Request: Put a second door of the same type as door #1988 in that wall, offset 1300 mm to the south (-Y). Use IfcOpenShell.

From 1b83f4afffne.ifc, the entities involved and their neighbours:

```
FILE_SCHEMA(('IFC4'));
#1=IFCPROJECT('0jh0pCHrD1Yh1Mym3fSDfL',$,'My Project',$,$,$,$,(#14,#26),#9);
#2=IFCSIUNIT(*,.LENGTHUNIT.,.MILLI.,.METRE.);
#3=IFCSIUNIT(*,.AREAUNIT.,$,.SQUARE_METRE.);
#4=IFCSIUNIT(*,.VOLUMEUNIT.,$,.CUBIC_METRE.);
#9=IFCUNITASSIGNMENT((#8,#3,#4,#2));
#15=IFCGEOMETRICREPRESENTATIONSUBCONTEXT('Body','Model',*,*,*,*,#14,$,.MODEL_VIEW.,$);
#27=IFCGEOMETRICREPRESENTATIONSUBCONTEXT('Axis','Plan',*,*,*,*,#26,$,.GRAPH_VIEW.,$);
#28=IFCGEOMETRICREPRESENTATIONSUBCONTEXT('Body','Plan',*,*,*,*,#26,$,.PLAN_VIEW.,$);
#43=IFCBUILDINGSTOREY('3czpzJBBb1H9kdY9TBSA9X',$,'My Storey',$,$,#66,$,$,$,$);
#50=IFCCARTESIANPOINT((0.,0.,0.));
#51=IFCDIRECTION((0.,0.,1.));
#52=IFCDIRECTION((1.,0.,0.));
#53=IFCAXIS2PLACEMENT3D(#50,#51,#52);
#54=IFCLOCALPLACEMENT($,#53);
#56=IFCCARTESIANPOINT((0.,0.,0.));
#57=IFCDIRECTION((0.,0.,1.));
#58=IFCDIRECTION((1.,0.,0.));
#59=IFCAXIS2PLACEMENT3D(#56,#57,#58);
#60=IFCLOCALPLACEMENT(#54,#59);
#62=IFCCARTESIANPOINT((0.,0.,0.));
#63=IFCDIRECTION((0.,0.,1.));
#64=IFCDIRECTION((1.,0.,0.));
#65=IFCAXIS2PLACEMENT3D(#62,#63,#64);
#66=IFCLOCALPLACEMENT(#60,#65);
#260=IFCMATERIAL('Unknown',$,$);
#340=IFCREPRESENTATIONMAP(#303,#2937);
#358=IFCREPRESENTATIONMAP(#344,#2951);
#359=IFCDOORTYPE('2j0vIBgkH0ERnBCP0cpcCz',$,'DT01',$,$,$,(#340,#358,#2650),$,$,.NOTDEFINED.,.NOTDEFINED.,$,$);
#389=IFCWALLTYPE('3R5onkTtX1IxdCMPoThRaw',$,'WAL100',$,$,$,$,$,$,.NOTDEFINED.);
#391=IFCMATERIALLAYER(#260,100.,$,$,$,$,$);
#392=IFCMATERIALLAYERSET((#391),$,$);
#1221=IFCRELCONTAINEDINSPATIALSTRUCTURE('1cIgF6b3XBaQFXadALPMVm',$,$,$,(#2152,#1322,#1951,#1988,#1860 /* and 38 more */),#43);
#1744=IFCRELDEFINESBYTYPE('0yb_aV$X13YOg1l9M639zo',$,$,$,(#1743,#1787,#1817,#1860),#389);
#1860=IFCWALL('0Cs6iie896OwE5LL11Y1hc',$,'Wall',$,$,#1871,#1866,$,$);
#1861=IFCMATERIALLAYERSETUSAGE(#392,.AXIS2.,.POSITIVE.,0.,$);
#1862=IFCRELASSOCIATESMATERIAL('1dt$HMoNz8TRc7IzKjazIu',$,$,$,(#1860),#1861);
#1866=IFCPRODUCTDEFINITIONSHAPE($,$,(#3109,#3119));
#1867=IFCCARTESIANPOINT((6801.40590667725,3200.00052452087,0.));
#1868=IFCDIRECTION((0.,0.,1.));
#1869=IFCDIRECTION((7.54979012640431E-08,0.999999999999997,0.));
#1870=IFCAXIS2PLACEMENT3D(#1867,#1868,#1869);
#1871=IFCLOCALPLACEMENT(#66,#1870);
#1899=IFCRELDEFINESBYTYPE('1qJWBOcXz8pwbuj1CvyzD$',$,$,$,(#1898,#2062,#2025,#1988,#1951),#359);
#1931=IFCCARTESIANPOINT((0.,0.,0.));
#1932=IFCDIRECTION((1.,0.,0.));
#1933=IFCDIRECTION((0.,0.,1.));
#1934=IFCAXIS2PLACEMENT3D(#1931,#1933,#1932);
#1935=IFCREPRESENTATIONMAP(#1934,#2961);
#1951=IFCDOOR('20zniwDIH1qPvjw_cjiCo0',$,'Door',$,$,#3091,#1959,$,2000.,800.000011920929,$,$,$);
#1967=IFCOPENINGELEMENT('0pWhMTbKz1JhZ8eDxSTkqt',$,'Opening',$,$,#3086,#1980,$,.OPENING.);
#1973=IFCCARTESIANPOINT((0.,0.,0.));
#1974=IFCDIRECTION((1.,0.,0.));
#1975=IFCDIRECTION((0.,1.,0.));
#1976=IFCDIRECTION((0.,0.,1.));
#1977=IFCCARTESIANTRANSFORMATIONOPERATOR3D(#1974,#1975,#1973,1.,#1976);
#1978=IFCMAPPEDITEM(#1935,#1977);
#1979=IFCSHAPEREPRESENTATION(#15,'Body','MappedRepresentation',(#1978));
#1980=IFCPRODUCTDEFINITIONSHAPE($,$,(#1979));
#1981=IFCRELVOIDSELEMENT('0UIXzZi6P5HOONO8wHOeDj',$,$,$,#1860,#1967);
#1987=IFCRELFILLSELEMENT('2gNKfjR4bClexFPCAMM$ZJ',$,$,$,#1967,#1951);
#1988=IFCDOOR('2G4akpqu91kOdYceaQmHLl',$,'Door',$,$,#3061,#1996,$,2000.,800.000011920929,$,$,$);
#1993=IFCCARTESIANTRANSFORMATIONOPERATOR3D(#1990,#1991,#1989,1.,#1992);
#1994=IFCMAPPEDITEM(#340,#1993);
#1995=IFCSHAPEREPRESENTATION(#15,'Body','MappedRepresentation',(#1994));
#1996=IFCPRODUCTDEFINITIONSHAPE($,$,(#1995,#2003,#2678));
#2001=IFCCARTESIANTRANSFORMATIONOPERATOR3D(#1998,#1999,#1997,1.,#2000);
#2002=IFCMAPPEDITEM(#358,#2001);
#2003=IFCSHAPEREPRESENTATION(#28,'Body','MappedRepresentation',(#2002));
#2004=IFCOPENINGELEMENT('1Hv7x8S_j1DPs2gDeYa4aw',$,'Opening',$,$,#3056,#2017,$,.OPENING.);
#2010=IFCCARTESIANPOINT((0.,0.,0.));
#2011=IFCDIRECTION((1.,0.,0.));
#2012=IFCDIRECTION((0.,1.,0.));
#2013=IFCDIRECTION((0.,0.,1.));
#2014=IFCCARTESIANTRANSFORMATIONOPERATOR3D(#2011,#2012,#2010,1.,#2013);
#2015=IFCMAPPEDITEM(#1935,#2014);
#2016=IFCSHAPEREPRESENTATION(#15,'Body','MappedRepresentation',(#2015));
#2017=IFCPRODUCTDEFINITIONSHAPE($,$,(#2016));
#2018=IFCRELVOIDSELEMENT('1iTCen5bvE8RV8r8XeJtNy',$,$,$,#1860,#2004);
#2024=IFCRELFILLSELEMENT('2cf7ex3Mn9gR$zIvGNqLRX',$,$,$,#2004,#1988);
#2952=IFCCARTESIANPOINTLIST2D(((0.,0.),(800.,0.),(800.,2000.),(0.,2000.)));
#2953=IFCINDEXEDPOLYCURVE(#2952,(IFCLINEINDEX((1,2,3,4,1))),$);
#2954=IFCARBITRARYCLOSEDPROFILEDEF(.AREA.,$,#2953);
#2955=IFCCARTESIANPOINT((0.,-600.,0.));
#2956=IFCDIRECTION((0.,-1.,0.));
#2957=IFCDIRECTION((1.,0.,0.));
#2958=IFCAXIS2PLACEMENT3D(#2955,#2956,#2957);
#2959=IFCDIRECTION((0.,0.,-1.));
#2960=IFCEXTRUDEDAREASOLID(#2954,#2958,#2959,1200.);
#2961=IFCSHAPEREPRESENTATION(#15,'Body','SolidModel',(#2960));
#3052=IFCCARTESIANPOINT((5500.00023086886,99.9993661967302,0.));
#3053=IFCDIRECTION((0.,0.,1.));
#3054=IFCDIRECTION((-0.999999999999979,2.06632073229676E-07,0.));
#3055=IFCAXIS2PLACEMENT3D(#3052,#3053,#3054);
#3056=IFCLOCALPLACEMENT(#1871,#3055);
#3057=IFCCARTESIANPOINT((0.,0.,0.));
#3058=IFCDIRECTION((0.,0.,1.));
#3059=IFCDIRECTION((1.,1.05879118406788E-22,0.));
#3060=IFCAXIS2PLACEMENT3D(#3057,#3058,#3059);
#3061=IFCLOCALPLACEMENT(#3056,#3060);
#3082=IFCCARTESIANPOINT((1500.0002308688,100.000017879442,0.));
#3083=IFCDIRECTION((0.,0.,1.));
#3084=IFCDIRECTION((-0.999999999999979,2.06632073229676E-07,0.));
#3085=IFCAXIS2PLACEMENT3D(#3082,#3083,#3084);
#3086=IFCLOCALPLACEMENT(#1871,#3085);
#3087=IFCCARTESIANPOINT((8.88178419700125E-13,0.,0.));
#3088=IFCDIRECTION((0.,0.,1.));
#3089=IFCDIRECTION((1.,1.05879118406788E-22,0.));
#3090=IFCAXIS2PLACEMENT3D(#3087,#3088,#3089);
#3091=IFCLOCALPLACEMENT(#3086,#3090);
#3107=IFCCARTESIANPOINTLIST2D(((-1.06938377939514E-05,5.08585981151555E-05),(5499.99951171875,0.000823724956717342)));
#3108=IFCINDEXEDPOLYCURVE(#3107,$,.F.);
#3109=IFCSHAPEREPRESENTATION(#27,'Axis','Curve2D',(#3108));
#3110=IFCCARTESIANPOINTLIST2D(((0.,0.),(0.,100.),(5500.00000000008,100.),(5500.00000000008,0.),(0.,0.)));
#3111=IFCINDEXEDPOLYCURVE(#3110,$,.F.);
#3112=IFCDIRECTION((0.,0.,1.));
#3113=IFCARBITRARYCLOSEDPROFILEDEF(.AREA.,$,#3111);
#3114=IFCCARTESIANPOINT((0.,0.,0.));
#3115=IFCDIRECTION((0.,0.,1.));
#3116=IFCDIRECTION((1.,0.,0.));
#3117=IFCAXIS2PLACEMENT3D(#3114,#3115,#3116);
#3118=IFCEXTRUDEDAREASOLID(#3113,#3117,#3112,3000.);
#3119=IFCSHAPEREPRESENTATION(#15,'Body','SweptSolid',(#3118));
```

```python
import ifcopenshell
import ifcopenshell.api.feature
import ifcopenshell.api.geometry
import ifcopenshell.api.root
import ifcopenshell.geom
import ifcopenshell.util.element
import ifcopenshell.util.placement
import ifcopenshell.util.shape

model = ifcopenshell.open("1b83f4afffne.ifc")
settings = ifcopenshell.geom.settings()


def volume(element):
    """Net volume in cubic metres, openings subtracted."""
    shape = ifcopenshell.geom.create_shape(settings, element)
    return ifcopenshell.util.shape.get_volume(shape.geometry)


door = model.by_id(1988)
opening = door.FillsVoids[0].RelatingOpeningElement
wall = opening.VoidsElements[0].RelatingBuildingElement
before = volume(wall)
shift = ifcopenshell.util.placement.get_local_placement(wall.ObjectPlacement)[:3, 0] * -1300.0

# copy_class copies the void relationship, type, container and properties, but no geometry.
new_opening = ifcopenshell.api.root.copy_class(model, product=opening)
new_opening.Representation = ifcopenshell.util.element.copy_deep(
    model, opening.Representation, exclude=["IfcGeometricRepresentationContext", "IfcRepresentationMap"]
)
new_door = ifcopenshell.api.root.copy_class(model, product=door)
new_door.Representation = ifcopenshell.util.element.copy_deep(
    model, door.Representation, exclude=["IfcGeometricRepresentationContext", "IfcRepresentationMap"]
)
ifcopenshell.api.feature.add_filling(model, opening=new_opening, element=new_door)

for old, new in ((opening, new_opening), (door, new_door)):
    matrix = ifcopenshell.util.placement.get_local_placement(old.ObjectPlacement)
    matrix[:3, 3] += shift
    ifcopenshell.api.geometry.edit_object_placement(model, product=new, matrix=matrix, is_si=False)

after = volume(wall)

print(f"wall volume {before:.3f} -> {after:.3f} m3")

model.write("1b83f4afffne_v2.ifc")
```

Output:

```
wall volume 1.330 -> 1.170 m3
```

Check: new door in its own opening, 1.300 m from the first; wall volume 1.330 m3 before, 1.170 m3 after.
